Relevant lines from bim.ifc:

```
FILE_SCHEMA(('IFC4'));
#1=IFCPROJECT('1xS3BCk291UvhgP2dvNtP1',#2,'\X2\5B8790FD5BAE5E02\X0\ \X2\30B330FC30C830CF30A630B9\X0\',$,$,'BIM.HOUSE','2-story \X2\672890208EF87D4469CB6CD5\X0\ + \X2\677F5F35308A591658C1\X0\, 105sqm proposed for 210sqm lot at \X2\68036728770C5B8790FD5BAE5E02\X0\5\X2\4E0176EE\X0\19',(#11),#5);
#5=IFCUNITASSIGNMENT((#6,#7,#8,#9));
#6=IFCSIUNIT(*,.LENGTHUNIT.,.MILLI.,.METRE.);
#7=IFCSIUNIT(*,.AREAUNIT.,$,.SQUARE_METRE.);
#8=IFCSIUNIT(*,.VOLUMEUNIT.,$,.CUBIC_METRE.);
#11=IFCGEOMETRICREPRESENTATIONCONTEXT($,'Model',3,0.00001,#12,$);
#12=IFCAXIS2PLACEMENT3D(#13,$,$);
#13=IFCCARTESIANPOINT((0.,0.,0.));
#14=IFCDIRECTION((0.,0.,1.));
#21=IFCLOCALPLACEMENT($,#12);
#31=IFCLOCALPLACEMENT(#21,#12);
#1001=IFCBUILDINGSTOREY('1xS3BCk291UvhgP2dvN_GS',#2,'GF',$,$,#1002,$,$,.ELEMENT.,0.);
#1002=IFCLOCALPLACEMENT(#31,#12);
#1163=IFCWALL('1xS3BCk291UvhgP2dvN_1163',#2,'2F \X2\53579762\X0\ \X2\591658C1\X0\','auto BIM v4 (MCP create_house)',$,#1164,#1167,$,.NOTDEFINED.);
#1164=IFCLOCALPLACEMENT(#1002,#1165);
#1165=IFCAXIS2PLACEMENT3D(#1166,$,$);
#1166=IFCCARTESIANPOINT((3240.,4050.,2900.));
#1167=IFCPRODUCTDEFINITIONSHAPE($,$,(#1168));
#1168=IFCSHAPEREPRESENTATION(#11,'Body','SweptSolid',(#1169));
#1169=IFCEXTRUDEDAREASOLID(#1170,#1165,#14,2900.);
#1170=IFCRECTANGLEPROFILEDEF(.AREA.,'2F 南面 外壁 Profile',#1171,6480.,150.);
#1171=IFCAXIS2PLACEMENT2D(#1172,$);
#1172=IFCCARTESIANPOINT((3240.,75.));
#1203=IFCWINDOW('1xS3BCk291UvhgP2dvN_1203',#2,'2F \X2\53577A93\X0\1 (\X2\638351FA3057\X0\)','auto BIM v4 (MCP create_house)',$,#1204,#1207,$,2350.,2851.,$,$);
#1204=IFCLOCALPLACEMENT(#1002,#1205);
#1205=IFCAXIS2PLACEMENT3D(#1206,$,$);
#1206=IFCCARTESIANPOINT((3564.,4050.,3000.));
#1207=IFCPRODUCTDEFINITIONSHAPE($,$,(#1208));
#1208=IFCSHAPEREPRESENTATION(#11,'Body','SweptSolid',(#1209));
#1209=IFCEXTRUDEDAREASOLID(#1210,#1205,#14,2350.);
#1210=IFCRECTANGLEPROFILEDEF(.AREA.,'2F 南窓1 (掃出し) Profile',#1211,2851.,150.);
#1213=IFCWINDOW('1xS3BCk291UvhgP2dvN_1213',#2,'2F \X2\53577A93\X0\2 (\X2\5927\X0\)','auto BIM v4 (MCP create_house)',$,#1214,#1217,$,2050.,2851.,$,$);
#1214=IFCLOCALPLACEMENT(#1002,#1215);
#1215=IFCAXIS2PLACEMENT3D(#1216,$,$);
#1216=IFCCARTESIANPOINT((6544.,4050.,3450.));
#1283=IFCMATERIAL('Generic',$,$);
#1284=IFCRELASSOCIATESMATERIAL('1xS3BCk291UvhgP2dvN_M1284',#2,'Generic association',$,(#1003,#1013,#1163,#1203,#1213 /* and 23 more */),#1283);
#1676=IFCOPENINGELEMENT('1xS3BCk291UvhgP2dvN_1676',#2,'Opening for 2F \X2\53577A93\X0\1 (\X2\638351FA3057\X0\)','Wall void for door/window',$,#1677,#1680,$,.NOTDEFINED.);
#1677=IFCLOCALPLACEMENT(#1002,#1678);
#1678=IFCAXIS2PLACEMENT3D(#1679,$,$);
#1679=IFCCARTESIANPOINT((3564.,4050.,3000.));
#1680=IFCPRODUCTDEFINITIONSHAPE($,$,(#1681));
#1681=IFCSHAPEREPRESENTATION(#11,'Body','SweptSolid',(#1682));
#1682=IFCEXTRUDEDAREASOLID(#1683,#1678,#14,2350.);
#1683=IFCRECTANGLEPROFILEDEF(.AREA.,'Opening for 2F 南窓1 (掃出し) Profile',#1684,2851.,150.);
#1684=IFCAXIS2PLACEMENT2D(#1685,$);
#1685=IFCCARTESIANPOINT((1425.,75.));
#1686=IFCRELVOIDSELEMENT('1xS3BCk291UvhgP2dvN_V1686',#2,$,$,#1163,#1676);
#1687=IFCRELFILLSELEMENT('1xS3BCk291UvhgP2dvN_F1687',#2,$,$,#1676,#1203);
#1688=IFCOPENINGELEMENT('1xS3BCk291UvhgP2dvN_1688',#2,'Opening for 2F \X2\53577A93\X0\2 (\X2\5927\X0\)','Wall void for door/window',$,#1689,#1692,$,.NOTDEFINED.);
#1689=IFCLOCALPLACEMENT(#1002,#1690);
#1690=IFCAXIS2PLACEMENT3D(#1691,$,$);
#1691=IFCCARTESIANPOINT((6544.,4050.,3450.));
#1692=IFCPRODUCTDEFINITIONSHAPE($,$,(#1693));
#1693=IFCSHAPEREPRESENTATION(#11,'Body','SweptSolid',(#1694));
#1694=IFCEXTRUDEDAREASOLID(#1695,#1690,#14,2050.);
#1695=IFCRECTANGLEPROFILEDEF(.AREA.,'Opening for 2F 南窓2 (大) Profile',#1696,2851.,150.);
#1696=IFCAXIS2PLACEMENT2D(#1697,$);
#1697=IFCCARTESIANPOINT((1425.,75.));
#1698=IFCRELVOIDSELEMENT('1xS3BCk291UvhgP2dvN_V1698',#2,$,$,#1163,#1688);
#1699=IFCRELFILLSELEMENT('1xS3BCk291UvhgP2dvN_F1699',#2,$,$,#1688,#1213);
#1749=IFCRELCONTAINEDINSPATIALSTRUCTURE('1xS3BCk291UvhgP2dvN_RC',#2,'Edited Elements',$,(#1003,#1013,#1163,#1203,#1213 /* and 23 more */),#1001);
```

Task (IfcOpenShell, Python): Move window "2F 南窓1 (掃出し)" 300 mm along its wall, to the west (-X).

```python
import ifcopenshell
import ifcopenshell.api.geometry
import ifcopenshell.util.placement

model = ifcopenshell.open("bim.ifc")

window = model.by_guid("1xS3BCk291UvhgP2dvN_1203")
opening = window.FillsVoids[0].RelatingOpeningElement
wall = opening.VoidsElements[0].RelatingBuildingElement

wall_matrix = ifcopenshell.util.placement.get_local_placement(wall.ObjectPlacement)
shift = wall_matrix[:3, 0] * -300.0
before = ifcopenshell.util.placement.get_local_placement(window.ObjectPlacement)[:3, 3].copy()

# The window is not placed relative to its opening, so move both.
for product in (opening, window):
    matrix = ifcopenshell.util.placement.get_local_placement(product.ObjectPlacement)
    matrix[:3, 3] += shift
    ifcopenshell.api.geometry.edit_object_placement(model, product=product, matrix=matrix, is_si=False)

after = ifcopenshell.util.placement.get_local_placement(window.ObjectPlacement)[:3, 3]
print("window moved by", (after - before).round(3) + 0.0)

model.write("bim_updated.ifc")
```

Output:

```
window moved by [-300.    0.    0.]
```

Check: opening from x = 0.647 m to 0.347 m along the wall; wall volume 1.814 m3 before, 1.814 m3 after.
